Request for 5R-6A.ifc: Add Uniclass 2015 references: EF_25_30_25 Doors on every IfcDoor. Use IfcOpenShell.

First a look at what the model holds.

```python
import ifcopenshell

model = ifcopenshell.open("5R-6A.ifc")
print(model.schema)
print("classifications:", [c.Name for c in model.by_type("IfcClassification")])
for ifc_class in ("IfcDoor", "IfcRoof", "IfcStair", "IfcWall", "IfcWindow"):
    print(ifc_class, len(model.by_type(ifc_class)))
```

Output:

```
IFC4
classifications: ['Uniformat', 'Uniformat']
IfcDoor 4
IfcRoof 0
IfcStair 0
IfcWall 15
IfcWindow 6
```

```python
import ifcopenshell
import ifcopenshell.api.classification

model = ifcopenshell.open("5R-6A.ifc")

system = ifcopenshell.api.classification.add_classification(model, classification="Uniclass 2015")

codes = {
    "IfcDoor": ("EF_25_30_25", "Doors"),
}
for ifc_class, (code, name) in codes.items():
    products = model.by_type(ifc_class)
    ifcopenshell.api.classification.add_reference(
        model, products=products, classification=system, identification=code, name=name
    )
    print(code, len(products))

model.write("5R-6A-out.ifc")
```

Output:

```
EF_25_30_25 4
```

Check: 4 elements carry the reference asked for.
